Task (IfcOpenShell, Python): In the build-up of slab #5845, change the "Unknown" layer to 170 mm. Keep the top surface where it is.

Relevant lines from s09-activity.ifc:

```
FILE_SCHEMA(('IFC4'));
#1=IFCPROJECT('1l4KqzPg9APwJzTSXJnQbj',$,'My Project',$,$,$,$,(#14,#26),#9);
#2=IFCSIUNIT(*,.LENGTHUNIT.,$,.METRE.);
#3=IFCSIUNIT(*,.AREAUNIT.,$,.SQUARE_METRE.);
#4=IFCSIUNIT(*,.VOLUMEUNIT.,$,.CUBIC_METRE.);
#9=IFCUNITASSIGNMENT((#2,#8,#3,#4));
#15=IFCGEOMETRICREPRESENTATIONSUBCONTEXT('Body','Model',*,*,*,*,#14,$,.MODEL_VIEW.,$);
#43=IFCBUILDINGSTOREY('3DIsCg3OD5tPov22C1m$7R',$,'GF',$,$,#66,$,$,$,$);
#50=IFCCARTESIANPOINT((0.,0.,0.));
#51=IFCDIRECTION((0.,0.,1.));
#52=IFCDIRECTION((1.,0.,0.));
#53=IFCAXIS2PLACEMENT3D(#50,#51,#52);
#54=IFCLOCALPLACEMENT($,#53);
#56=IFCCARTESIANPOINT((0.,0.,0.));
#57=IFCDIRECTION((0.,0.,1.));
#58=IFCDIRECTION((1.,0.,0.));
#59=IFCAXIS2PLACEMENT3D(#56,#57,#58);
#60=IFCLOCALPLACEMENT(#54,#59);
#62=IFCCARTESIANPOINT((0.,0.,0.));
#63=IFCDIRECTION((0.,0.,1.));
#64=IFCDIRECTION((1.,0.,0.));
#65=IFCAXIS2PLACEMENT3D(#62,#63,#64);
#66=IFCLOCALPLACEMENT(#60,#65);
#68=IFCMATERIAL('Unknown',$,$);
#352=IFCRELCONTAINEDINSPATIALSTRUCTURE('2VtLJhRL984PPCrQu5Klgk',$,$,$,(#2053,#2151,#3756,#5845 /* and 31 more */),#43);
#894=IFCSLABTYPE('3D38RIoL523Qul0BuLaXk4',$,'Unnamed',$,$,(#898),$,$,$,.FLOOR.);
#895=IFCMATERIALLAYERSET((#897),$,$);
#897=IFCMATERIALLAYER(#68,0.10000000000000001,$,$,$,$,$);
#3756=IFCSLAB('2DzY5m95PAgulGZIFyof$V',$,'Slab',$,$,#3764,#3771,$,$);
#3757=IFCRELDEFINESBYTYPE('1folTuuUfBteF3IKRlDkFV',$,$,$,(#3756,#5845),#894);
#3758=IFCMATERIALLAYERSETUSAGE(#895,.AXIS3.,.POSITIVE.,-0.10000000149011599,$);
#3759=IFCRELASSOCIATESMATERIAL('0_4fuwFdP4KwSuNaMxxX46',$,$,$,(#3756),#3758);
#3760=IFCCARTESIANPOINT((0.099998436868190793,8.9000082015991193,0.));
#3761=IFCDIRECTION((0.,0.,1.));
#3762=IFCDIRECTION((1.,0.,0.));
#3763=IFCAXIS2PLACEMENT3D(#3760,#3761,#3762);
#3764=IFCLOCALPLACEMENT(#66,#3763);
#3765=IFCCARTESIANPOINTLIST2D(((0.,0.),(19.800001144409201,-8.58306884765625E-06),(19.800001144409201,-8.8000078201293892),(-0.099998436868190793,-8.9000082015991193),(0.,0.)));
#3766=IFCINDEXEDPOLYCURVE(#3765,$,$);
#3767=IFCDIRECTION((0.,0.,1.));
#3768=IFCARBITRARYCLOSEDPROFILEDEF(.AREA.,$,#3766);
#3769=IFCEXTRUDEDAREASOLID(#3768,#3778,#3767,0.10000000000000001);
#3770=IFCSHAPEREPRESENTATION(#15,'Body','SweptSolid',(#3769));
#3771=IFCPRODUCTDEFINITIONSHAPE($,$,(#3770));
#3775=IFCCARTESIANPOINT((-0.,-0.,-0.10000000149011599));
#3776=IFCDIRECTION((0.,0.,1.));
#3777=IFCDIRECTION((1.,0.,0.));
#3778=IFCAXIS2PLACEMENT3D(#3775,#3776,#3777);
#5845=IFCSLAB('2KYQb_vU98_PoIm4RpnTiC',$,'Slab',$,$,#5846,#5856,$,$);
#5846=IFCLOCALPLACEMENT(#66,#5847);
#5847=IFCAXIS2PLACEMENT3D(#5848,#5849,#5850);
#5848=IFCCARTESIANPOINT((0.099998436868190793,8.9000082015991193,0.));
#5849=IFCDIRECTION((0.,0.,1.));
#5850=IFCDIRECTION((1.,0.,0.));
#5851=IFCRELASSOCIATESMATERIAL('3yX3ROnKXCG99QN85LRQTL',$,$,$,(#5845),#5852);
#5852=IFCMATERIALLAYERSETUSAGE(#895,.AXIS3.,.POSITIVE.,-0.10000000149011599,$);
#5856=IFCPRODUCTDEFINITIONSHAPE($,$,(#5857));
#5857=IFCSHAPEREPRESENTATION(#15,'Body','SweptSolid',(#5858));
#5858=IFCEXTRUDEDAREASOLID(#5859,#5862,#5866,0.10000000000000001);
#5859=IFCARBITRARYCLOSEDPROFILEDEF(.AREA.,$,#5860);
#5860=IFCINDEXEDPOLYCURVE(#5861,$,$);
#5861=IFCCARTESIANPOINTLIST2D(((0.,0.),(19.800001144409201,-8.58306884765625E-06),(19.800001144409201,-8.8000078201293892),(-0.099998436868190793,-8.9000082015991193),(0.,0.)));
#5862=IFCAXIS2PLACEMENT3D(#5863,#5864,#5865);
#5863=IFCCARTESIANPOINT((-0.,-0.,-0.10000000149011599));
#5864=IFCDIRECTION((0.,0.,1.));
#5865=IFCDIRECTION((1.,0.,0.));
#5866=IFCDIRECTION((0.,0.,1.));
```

```python
import ifcopenshell
import ifcopenshell.util.element
import ifcopenshell.util.representation

model = ifcopenshell.open("s09-activity.ifc")

layer_set = model.by_id(895)
layer = next(l for l in layer_set.MaterialLayers if l.Material and l.Material.Name == "Unknown")
change = 0.17 - layer.LayerThickness
layer.LayerThickness += change

# The layer set is shared, so every slab that uses it gets the new thickness.
slabs = [e for e in ifcopenshell.util.element.get_elements_by_material(model, layer_set) if e.is_a("IfcSlab")]
for slab in sorted(slabs, key=lambda e: e.id()):
    body = ifcopenshell.util.representation.get_representation(slab, "Model", "Body")
    solid = body.Items[0]
    old_depth = solid.Depth
    solid.Depth += change
    # Extruded upwards: lower the start of the extrusion so the top stays.
    x, y, z = solid.Position.Location.Coordinates
    solid.Position.Location = model.createIfcCartesianPoint((x, y, z - change))
    print(slab.id(), f"{old_depth:g} -> {solid.Depth:g}")

# The layers are counted up from the underside, which has moved.
for usage in {ifcopenshell.util.element.get_material(slab) for slab in slabs}:
    usage.OffsetFromReferenceLine -= change

model.write("s09-activity_updated.ifc")
```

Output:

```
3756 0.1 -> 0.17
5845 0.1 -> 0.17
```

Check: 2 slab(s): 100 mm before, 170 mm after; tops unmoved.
